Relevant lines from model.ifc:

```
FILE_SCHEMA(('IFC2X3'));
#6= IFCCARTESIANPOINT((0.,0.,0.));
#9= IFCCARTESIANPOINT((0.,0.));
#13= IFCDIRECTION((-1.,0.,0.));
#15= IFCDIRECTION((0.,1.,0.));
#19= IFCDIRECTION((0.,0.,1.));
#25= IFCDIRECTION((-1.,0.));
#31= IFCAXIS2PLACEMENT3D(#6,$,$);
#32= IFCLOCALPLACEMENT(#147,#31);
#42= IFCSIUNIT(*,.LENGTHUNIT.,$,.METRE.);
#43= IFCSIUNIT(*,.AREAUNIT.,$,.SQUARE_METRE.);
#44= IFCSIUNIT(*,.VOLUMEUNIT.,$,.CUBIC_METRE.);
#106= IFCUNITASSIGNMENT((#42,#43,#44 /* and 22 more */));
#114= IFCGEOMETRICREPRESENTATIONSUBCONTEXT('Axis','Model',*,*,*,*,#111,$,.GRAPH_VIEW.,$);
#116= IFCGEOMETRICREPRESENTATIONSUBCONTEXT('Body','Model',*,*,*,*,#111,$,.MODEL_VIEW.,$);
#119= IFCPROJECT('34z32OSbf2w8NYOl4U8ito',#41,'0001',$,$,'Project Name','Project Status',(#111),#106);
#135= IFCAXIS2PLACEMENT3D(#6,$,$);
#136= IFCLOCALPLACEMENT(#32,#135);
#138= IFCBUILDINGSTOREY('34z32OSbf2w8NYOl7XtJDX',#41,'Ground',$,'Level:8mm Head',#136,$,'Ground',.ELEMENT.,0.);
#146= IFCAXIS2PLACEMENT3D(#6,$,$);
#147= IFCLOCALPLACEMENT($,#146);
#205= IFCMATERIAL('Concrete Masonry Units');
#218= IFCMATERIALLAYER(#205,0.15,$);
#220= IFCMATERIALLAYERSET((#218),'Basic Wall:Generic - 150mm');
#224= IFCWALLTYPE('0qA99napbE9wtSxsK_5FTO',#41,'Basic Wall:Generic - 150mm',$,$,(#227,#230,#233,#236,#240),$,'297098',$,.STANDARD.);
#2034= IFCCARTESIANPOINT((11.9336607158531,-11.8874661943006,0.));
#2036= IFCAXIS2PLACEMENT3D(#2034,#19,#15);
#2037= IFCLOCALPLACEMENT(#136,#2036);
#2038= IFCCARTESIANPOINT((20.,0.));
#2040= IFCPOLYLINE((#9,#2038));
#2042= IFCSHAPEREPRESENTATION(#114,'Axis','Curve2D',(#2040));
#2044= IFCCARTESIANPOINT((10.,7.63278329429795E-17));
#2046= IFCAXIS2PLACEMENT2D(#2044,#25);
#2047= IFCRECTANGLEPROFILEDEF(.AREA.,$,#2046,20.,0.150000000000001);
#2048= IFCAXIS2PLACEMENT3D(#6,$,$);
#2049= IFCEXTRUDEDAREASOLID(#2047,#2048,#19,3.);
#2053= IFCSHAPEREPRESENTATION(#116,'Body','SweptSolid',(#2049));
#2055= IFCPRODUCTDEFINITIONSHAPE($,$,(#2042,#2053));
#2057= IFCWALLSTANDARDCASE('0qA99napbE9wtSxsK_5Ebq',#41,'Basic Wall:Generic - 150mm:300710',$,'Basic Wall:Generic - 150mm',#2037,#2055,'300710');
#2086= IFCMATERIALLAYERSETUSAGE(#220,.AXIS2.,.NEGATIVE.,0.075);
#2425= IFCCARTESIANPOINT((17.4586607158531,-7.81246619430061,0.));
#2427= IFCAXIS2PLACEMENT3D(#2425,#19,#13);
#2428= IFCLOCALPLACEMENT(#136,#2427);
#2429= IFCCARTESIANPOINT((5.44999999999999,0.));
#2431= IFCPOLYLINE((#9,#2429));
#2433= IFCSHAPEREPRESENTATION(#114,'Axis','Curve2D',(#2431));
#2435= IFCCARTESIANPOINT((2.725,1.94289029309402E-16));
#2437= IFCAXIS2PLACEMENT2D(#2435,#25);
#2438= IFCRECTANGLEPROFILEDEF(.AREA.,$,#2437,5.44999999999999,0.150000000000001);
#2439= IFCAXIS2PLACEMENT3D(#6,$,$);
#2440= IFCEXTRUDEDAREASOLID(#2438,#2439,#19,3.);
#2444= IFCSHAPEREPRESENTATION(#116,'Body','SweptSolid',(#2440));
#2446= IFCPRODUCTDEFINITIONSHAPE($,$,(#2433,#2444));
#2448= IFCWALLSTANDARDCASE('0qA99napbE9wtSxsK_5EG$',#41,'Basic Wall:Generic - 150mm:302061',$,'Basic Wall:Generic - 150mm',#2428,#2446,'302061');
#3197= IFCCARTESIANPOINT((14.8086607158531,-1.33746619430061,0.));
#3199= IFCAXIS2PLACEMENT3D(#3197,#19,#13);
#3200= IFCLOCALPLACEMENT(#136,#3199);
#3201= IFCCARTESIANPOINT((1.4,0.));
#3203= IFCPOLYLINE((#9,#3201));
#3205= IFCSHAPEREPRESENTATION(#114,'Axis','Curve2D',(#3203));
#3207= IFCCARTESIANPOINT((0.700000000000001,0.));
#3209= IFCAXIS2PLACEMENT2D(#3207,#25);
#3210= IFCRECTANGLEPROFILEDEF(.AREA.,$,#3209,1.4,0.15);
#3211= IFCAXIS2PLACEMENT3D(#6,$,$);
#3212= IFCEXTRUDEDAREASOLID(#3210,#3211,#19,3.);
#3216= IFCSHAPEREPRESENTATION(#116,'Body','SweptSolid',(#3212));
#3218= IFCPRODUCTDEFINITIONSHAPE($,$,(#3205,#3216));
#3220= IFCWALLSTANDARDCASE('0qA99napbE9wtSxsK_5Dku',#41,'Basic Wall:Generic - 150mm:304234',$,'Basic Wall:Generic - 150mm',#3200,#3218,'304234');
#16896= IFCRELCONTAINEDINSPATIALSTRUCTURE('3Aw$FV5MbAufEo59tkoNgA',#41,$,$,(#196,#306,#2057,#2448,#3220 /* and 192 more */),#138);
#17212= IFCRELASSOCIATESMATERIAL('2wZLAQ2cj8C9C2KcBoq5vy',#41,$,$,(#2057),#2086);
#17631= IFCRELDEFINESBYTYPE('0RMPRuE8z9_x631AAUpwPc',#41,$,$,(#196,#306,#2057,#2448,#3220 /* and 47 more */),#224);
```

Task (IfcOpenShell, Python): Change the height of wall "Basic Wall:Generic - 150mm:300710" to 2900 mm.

```python
import ifcopenshell
import ifcopenshell.geom
import ifcopenshell.util.representation
import ifcopenshell.util.shape
import ifcopenshell.util.unit

model = ifcopenshell.open("model.ifc")
unit_scale = ifcopenshell.util.unit.calculate_unit_scale(model)
settings = ifcopenshell.geom.settings()


def volume(element):
    """Net volume in cubic metres, openings subtracted."""
    shape = ifcopenshell.geom.create_shape(settings, element)
    return ifcopenshell.util.shape.get_volume(shape.geometry)


wall = model.by_guid("0qA99napbE9wtSxsK_5Ebq")
before = volume(wall)

body = ifcopenshell.util.representation.get_representation(wall, "Model", "Body")
solid = body.Items[0]
old_height = solid.Depth
solid.Depth = 2.9 / unit_scale
after = volume(wall)

print(f"height {old_height:g} -> {solid.Depth:g}, volume {before:.3f} -> {after:.3f} m3")

model.write("model-out.ifc")
```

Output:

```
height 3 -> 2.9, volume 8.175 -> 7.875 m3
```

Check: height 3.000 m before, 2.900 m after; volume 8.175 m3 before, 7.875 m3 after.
